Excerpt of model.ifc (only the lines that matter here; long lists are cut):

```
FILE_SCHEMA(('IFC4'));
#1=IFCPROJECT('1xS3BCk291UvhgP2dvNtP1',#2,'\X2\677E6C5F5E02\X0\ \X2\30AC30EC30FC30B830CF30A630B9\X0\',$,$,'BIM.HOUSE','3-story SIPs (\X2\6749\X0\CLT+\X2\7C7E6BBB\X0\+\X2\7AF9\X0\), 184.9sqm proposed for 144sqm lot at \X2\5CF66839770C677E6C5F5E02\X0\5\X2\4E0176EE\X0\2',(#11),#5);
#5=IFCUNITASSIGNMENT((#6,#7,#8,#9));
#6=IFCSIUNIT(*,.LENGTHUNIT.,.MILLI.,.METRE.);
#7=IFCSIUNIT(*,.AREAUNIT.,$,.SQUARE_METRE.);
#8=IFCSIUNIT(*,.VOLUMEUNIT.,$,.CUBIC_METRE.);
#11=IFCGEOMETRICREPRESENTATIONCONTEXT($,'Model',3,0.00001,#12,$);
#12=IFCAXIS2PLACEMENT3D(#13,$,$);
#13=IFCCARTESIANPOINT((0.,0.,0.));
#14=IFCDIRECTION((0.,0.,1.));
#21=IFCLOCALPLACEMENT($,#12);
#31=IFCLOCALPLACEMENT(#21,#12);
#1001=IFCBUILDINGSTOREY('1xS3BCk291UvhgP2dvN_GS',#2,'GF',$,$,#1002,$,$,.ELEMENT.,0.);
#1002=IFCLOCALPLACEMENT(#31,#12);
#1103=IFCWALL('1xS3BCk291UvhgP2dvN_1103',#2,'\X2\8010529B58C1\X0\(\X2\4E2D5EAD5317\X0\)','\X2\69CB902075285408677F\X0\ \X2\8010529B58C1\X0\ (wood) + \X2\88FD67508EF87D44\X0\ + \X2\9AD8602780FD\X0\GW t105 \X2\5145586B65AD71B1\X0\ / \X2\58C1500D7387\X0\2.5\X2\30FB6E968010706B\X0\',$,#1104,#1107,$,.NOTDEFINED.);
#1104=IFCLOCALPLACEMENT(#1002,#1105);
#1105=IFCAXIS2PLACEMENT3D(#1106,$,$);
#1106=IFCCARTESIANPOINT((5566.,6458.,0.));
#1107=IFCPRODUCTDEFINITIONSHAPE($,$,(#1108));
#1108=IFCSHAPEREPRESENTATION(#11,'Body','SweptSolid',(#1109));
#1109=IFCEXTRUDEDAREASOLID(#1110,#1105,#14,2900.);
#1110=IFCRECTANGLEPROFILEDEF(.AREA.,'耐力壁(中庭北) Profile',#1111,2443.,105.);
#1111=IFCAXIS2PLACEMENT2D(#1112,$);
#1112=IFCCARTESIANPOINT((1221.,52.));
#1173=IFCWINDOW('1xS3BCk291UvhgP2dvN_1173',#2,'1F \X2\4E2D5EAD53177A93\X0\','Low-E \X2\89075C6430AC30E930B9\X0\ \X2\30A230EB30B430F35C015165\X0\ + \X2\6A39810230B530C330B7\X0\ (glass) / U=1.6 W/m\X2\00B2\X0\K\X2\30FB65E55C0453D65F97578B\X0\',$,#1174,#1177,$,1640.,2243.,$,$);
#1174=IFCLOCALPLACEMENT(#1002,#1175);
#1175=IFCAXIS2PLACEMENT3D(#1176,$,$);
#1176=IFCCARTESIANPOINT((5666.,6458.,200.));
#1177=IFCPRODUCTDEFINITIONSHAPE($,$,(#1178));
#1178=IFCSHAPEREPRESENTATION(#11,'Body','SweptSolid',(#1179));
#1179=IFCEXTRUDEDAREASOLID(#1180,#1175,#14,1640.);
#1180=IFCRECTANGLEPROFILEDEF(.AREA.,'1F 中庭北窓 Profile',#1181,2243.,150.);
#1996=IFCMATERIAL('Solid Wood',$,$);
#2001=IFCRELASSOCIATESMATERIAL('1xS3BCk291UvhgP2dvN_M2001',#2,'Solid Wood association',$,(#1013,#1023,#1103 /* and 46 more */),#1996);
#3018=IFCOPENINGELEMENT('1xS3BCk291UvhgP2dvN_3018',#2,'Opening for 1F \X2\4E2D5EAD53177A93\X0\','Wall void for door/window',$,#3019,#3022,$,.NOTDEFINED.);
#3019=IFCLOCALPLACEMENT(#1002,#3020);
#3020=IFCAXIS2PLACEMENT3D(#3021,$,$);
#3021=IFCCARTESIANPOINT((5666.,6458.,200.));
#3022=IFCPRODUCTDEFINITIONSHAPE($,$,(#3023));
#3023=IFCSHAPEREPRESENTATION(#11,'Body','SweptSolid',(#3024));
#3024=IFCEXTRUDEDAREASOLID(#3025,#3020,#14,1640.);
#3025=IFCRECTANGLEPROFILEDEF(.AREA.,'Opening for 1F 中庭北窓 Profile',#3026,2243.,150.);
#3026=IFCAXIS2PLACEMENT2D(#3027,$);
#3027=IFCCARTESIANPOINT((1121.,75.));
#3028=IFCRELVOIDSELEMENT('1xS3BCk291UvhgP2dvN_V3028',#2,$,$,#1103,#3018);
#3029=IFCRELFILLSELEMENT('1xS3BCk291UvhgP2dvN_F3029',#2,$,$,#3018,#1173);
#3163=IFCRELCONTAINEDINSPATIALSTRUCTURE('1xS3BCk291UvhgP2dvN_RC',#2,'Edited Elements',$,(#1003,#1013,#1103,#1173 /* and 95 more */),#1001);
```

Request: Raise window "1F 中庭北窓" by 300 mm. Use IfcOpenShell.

```python
import numpy as np
import ifcopenshell
import ifcopenshell.api.geometry
import ifcopenshell.util.placement
import ifcopenshell.util.unit

model = ifcopenshell.open("model.ifc")
unit_scale = ifcopenshell.util.unit.calculate_unit_scale(model)

window = model.by_guid("1xS3BCk291UvhgP2dvN_1173")
opening = window.FillsVoids[0].RelatingOpeningElement
dz = 0.3 / unit_scale

shift = np.array([0.0, 0.0, dz])
# The window is not placed relative to its opening, so move both.
for product in (opening, window):
    matrix = ifcopenshell.util.placement.get_local_placement(product.ObjectPlacement)
    matrix[:3, 3] += shift
    ifcopenshell.api.geometry.edit_object_placement(model, product=product, matrix=matrix, is_si=False)

print(f"moved by {dz * unit_scale:+.3f} m")

model.write("model_edited.ifc")
```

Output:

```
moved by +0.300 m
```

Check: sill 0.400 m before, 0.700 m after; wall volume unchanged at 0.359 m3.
